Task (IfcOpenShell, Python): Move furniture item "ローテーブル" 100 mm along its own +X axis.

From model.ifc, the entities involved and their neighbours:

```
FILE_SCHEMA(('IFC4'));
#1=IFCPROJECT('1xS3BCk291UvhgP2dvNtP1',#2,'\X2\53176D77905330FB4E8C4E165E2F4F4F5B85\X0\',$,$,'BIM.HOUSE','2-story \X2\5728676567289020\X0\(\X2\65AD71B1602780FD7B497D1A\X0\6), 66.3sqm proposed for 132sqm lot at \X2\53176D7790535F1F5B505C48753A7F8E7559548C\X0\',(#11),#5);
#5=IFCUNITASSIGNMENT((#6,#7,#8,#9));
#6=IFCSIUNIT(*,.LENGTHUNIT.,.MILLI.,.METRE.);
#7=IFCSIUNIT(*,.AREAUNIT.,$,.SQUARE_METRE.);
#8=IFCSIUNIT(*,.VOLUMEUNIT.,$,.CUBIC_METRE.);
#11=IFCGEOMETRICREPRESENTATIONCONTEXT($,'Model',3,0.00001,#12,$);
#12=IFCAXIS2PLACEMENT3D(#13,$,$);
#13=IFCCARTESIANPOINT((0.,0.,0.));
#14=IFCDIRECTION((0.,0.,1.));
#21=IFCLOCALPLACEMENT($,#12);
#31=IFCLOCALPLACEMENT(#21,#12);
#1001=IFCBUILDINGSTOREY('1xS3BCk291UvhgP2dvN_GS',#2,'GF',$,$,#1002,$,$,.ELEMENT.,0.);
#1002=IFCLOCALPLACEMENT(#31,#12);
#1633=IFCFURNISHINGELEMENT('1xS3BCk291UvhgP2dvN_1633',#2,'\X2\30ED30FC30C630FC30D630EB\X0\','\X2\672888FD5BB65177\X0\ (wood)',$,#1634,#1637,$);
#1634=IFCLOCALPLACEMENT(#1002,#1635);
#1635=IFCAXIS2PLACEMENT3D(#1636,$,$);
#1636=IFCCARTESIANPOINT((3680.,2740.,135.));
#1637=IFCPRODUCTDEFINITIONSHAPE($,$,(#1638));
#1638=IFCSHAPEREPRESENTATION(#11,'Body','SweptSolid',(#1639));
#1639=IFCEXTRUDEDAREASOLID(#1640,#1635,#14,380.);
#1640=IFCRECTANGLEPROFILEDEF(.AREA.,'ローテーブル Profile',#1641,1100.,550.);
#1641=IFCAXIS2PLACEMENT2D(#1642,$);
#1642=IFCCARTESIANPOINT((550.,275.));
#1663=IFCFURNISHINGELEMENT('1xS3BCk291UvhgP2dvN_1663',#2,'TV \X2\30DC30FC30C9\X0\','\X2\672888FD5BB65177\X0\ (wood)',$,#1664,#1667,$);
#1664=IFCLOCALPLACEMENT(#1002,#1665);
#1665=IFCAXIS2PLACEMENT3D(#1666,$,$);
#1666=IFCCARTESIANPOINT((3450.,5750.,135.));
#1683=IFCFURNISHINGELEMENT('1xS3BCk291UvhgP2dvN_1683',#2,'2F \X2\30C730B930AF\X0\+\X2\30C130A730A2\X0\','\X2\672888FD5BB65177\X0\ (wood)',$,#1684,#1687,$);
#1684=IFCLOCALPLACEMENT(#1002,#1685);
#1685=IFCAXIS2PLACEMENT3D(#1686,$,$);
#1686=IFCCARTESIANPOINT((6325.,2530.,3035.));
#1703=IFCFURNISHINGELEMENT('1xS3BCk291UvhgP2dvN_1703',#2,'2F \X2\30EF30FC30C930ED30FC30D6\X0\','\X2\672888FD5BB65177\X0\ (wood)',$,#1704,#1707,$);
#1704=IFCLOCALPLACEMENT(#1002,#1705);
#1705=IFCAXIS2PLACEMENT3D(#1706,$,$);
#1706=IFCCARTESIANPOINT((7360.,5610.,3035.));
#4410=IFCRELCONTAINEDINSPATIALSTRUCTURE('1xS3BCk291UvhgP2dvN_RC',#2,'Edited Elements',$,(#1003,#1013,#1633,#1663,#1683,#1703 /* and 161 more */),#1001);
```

```python
import ifcopenshell
import ifcopenshell.api.geometry
import ifcopenshell.util.placement

model = ifcopenshell.open("model.ifc")

item = model.by_id(1633)
matrix = ifcopenshell.util.placement.get_local_placement(item.ObjectPlacement)
matrix[:3, 3] += matrix[:3, 0] * 100.0
ifcopenshell.api.geometry.edit_object_placement(model, product=item, matrix=matrix, is_si=False)

print(ifcopenshell.util.placement.get_local_placement(item.ObjectPlacement).round(3) + 0.0)

model.write("model_edited.ifc")
```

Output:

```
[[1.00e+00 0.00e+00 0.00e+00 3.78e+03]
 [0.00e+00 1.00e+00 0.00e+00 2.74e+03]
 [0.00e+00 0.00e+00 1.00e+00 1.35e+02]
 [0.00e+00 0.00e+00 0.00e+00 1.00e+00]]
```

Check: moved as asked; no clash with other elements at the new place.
